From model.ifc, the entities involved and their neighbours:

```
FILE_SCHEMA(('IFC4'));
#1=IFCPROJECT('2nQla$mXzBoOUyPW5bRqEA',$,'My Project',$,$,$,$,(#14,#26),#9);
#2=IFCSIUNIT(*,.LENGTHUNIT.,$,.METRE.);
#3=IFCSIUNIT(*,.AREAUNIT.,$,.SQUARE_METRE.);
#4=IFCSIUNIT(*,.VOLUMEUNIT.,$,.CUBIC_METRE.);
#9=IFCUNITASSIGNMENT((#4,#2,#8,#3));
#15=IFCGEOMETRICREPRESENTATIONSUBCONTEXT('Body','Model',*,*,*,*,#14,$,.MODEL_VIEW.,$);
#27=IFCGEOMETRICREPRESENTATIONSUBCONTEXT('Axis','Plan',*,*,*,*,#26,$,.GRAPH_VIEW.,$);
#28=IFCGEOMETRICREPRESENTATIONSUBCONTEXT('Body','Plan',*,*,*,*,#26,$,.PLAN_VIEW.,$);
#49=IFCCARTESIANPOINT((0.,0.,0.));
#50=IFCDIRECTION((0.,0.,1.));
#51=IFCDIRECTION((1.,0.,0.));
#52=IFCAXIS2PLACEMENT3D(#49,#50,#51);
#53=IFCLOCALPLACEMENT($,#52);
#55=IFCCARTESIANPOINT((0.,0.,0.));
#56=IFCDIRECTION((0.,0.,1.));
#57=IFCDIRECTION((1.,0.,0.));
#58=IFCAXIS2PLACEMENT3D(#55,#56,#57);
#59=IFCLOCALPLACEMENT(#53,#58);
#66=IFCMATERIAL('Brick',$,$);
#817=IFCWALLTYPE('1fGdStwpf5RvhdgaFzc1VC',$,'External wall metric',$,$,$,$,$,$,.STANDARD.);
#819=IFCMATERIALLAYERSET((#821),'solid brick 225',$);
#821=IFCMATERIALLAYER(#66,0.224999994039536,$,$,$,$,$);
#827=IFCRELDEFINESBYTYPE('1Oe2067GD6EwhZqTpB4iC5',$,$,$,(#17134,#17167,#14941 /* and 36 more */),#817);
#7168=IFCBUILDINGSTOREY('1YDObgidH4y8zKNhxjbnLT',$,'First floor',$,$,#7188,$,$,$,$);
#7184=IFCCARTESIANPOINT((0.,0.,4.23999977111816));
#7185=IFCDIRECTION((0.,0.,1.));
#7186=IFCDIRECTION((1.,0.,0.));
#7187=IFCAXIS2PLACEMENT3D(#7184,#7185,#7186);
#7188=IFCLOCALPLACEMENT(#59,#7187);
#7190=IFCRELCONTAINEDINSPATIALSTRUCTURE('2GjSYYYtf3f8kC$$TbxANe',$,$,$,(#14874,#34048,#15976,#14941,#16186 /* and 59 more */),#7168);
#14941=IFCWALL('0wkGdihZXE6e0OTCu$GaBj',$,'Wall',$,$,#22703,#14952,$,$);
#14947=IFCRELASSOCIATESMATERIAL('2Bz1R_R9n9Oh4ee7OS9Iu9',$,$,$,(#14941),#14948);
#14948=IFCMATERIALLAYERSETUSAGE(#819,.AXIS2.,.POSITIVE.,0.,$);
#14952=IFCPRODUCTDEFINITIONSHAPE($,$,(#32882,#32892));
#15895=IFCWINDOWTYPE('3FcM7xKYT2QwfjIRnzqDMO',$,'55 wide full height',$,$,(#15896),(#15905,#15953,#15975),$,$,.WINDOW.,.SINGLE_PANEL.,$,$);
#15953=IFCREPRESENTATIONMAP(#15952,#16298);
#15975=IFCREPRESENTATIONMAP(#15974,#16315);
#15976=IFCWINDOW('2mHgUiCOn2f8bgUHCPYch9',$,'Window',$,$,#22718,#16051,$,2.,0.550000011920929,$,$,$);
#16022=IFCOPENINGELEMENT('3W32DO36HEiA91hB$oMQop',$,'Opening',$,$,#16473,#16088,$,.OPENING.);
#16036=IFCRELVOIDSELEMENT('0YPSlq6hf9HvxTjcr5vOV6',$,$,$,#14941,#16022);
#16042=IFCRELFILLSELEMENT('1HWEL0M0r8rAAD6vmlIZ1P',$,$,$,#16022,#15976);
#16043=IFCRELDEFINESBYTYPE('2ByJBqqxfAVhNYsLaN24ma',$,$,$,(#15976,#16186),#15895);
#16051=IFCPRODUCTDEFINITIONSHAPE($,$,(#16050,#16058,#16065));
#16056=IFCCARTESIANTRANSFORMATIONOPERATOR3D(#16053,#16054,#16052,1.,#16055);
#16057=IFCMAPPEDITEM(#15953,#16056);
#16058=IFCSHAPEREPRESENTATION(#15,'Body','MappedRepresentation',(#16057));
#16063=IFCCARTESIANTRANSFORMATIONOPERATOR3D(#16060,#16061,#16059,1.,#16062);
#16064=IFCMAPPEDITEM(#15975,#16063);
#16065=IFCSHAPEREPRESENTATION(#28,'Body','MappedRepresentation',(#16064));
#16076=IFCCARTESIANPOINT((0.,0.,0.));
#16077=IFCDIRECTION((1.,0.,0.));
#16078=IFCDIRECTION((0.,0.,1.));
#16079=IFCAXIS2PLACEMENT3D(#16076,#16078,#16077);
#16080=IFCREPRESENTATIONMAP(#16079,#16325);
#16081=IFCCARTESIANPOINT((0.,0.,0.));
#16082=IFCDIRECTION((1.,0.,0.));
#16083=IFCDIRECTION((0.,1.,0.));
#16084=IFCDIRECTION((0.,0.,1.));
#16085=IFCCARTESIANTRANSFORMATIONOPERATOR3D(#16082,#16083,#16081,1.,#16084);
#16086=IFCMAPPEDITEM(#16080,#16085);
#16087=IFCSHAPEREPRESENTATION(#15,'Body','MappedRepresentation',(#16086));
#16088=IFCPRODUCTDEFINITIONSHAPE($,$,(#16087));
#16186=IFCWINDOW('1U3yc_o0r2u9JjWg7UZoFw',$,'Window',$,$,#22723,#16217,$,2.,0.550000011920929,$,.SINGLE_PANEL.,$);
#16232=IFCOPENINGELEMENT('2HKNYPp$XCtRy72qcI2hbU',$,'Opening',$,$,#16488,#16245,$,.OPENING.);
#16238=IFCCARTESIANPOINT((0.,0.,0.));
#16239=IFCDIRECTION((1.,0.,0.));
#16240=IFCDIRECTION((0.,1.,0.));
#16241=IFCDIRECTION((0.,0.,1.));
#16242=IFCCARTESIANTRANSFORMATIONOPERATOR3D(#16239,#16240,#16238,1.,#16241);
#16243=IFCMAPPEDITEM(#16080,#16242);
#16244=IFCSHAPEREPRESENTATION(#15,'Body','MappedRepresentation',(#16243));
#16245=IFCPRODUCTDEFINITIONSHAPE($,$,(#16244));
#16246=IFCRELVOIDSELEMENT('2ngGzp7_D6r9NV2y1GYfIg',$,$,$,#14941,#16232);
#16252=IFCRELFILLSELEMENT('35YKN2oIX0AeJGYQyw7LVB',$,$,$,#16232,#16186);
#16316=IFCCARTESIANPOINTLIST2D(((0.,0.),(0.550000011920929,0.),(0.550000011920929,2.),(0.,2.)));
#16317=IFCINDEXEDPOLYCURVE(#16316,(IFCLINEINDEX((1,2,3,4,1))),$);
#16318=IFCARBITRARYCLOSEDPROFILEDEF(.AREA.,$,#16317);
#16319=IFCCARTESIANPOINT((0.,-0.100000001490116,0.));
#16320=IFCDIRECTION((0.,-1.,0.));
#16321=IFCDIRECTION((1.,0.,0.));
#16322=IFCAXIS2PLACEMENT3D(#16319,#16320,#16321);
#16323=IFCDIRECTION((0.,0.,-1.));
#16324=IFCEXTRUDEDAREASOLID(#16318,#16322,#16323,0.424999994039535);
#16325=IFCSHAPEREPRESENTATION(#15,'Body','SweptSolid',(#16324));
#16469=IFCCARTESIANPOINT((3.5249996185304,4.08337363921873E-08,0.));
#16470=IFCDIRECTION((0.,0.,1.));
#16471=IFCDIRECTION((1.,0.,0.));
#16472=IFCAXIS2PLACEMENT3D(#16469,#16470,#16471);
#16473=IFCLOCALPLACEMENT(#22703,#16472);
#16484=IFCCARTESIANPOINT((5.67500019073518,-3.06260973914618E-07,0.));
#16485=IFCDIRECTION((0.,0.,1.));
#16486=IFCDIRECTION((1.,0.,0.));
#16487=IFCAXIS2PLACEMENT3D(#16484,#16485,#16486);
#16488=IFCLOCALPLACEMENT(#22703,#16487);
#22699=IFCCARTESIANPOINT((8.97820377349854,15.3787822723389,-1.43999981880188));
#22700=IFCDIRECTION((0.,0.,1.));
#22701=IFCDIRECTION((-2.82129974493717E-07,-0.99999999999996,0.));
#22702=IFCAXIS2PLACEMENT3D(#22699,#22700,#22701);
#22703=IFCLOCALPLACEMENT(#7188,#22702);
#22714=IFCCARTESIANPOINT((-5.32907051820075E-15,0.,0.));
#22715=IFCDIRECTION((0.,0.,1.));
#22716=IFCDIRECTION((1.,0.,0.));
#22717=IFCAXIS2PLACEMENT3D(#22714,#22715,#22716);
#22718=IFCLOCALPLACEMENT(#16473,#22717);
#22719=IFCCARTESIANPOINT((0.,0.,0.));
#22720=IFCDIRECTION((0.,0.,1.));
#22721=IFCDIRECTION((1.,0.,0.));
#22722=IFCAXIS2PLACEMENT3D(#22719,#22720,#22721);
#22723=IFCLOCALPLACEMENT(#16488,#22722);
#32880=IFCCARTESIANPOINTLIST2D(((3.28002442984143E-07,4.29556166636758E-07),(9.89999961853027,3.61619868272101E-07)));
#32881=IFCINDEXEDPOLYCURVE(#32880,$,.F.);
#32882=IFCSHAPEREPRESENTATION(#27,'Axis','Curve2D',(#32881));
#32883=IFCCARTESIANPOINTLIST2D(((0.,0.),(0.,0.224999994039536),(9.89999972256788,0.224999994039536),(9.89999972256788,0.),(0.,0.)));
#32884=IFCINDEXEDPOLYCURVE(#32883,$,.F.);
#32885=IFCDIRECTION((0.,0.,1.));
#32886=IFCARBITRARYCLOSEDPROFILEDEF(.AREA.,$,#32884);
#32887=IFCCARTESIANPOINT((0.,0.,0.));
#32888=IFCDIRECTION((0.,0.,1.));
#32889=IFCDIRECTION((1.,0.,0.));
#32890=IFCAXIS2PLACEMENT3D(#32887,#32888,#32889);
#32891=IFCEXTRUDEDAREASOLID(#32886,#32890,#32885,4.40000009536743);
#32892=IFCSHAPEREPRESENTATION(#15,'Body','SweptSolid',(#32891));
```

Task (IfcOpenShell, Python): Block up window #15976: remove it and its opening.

```python
import ifcopenshell
import ifcopenshell.api.feature
import ifcopenshell.api.root
import ifcopenshell.geom
import ifcopenshell.util.shape

model = ifcopenshell.open("model.ifc")
settings = ifcopenshell.geom.settings()


def volume(element):
    """Net volume in cubic metres, openings subtracted."""
    shape = ifcopenshell.geom.create_shape(settings, element)
    return ifcopenshell.util.shape.get_volume(shape.geometry)


window = model.by_guid("2mHgUiCOn2f8bgUHCPYch9")
opening = window.FillsVoids[0].RelatingOpeningElement
wall = opening.VoidsElements[0].RelatingBuildingElement
before = volume(wall)

ifcopenshell.api.root.remove_product(model, product=window)
ifcopenshell.api.feature.remove_feature(model, feature=opening)

after = volume(wall)

print(f"wall volume {before:.3f} -> {after:.3f} m3")

model.write("model_rev.ifc")
```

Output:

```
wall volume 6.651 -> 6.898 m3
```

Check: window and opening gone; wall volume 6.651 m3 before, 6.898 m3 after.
